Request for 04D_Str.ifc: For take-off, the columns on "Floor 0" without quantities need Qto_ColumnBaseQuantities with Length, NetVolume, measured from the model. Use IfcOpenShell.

First a look at what the model holds.

```python
import ifcopenshell
import ifcopenshell.util.element
import ifcopenshell.util.unit

model = ifcopenshell.open("04D_Str.ifc")
print(model.schema)
for unit_type in ("LENGTHUNIT", "AREAUNIT", "VOLUMEUNIT"):
    print(unit_type, ifcopenshell.util.unit.calculate_unit_scale(model, unit_type))
storey = next(s for s in model.by_type("IfcBuildingStorey") if s.Name == "Floor 0")
columns = [e for e in ifcopenshell.util.element.get_decomposition(storey) if e.is_a("IfcColumn")]
for e in sorted(columns, key=lambda e: e.id()):
    print(e.id(), e.is_a(), e.Name, list(ifcopenshell.util.element.get_psets(e, qtos_only=True)), sep=" | ")
```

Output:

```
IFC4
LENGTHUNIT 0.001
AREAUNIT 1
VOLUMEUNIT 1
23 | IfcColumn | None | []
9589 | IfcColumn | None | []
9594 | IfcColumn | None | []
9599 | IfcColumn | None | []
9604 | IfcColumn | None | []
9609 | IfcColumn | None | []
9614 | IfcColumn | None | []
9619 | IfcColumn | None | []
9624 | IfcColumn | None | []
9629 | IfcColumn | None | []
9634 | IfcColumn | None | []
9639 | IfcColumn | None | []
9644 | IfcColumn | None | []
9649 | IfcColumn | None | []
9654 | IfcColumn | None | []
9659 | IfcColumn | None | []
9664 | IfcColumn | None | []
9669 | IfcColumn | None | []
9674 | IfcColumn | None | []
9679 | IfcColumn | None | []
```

```python
import ifcopenshell
import ifcopenshell.api.pset
import ifcopenshell.geom
import ifcopenshell.util.element
import ifcopenshell.util.shape
import ifcopenshell.util.unit

model = ifcopenshell.open("04D_Str.ifc")
unit_scale = ifcopenshell.util.unit.calculate_unit_scale(model)
volume_scale = ifcopenshell.util.unit.calculate_unit_scale(model, "VOLUMEUNIT")
settings = ifcopenshell.geom.settings()

storey = next(s for s in model.by_type("IfcBuildingStorey") if s.Name == "Floor 0")
columns = [e for e in ifcopenshell.util.element.get_decomposition(storey) if e.is_a("IfcColumn")]

for e in sorted(columns, key=lambda e: e.id()):
    if ifcopenshell.util.element.get_psets(e, qtos_only=True, should_inherit=False):
        continue
    # Geometry comes back in metres, in the element's own axes.
    shape = ifcopenshell.geom.create_shape(settings, e)
    values = {
        "Length": ifcopenshell.util.shape.get_z(shape.geometry) / unit_scale,
        "NetVolume": ifcopenshell.util.shape.get_volume(shape.geometry) / volume_scale,
    }
    qto = ifcopenshell.api.pset.add_qto(model, product=e, name="Qto_ColumnBaseQuantities")
    ifcopenshell.api.pset.edit_qto(model, qto=qto, properties=values)
    print(e.id(), {k: round(v, 3) for k, v in values.items()})

model.write("04D_Str_edited.ifc")
```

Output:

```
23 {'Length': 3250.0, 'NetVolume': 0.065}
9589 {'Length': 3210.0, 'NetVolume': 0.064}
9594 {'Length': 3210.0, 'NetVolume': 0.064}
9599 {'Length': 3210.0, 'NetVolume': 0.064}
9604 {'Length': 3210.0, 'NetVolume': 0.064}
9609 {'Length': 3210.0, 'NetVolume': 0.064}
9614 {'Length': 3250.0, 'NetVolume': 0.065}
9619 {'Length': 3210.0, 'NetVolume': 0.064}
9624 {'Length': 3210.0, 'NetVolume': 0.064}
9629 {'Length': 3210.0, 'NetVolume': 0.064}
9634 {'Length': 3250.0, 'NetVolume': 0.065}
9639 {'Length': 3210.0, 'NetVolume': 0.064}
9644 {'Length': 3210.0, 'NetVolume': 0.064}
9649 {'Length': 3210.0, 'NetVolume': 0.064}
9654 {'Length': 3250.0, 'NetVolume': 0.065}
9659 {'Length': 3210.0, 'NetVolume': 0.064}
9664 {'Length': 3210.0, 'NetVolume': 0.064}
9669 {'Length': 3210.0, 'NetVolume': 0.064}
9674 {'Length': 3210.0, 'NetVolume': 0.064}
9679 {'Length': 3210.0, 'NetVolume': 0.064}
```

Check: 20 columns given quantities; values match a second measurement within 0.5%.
